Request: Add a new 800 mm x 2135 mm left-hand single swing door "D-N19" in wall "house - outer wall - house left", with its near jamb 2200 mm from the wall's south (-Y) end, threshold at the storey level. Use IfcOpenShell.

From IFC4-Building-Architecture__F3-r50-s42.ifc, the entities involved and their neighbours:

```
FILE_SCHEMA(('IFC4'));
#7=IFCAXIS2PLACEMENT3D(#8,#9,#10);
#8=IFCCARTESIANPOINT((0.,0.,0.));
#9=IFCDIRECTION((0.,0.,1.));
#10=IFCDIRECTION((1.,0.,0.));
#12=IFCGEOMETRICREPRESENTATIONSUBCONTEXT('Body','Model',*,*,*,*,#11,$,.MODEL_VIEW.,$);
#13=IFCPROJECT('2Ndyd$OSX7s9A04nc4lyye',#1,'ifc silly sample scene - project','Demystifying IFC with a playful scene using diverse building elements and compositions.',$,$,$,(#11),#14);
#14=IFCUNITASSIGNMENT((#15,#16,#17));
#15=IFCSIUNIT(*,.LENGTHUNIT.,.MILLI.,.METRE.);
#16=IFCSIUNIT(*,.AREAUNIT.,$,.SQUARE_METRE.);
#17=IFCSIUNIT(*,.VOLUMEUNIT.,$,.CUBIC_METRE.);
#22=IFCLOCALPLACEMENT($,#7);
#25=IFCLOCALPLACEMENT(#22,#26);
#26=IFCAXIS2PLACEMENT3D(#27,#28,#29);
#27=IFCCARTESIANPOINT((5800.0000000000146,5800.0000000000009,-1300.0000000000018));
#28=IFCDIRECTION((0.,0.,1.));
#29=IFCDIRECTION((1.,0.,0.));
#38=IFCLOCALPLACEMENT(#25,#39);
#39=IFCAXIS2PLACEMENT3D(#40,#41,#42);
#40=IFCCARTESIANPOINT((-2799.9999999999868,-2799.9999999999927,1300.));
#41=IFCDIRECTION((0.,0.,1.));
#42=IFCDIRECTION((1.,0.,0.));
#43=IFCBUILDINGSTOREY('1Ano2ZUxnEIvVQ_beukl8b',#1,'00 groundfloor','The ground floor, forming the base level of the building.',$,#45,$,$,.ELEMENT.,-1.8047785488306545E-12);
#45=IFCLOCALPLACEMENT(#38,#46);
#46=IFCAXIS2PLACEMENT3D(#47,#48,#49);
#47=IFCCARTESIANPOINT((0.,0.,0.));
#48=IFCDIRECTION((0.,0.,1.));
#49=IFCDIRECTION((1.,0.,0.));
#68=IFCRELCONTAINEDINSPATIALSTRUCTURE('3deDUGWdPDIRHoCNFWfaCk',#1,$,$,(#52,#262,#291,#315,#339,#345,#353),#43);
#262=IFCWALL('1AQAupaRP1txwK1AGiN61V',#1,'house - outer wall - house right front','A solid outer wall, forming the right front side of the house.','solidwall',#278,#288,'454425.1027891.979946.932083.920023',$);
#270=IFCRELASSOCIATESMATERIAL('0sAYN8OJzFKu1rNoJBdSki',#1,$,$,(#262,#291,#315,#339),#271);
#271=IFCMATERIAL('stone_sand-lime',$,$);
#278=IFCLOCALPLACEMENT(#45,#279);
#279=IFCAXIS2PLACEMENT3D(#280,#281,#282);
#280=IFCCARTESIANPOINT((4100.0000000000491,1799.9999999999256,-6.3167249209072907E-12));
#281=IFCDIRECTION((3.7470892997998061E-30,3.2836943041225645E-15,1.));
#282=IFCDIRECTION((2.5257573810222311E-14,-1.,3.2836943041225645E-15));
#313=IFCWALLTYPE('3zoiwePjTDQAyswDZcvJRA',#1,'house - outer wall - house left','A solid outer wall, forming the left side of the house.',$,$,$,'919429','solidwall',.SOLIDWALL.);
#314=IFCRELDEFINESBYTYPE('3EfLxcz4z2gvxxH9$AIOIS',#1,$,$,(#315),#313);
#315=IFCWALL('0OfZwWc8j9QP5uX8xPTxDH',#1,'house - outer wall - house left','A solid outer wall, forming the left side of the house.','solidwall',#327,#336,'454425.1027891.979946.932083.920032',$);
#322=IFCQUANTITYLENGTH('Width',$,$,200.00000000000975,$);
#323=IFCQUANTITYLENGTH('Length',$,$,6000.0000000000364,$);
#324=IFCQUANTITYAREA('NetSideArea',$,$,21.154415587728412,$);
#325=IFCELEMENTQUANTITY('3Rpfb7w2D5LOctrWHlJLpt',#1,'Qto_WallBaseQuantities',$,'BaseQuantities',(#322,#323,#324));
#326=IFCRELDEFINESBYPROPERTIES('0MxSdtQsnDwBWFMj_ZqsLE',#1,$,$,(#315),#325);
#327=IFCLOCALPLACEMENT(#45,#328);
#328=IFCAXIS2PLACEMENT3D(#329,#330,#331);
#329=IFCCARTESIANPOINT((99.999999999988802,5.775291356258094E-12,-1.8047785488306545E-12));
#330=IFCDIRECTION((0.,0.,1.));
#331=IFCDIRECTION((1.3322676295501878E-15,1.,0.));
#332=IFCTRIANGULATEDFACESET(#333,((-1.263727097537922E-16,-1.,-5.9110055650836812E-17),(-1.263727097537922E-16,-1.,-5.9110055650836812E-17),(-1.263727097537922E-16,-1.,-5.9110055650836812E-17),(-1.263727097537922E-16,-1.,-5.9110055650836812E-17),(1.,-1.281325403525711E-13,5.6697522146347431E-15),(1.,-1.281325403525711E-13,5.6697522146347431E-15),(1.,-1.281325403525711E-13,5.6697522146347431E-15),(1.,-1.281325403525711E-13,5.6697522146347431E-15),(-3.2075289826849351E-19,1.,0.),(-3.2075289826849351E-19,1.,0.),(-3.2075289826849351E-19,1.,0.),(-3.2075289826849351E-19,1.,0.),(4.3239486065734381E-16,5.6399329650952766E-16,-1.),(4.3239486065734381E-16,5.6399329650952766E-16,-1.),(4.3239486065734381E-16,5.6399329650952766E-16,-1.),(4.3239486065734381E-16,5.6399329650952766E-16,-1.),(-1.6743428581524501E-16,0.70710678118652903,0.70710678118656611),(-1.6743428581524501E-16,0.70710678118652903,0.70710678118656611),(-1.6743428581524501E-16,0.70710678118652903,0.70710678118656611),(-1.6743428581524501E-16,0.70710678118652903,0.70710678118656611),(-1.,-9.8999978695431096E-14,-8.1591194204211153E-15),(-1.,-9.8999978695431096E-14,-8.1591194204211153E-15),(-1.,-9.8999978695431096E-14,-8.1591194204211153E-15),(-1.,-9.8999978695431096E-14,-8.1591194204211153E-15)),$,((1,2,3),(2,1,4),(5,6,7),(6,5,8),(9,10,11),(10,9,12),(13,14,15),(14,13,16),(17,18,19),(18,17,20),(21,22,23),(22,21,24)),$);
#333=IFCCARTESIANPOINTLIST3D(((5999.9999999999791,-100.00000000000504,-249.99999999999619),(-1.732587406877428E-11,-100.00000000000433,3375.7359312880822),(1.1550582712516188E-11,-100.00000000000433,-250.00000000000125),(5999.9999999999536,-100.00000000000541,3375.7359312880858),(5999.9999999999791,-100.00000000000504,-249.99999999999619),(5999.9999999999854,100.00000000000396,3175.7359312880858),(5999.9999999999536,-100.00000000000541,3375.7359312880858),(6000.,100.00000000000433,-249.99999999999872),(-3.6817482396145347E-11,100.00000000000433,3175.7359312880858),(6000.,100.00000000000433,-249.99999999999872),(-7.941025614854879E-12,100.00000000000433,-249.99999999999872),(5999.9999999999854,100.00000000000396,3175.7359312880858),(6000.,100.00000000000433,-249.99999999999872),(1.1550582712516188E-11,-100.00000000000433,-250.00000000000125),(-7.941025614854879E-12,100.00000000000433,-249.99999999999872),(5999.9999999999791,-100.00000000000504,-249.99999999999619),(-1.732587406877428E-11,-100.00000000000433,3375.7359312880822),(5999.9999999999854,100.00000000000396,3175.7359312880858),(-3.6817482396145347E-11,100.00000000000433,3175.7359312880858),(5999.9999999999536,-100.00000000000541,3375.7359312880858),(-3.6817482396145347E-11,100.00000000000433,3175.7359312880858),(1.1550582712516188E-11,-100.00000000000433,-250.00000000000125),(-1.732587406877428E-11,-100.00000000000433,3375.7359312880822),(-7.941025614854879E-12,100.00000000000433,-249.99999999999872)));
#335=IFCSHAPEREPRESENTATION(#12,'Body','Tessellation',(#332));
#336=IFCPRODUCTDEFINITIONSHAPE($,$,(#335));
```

```python
import numpy as np
import ifcopenshell
import ifcopenshell.api.feature
import ifcopenshell.api.geometry
import ifcopenshell.api.pset
import ifcopenshell.api.root
import ifcopenshell.api.spatial
import ifcopenshell.geom
import ifcopenshell.util.element
import ifcopenshell.util.placement
import ifcopenshell.util.representation
import ifcopenshell.util.shape
import ifcopenshell.util.unit

model = ifcopenshell.open("IFC4-Building-Architecture__F3-r50-s42.ifc")
unit_scale = ifcopenshell.util.unit.calculate_unit_scale(model)
area_scale = ifcopenshell.util.unit.calculate_unit_scale(model, "AREAUNIT")
settings = ifcopenshell.geom.settings()


def volume(element):
    """Net volume in cubic metres, openings subtracted."""
    shape = ifcopenshell.geom.create_shape(settings, element)
    return ifcopenshell.util.shape.get_volume(shape.geometry)


wall = model.by_guid("0OfZwWc8j9QP5uX8xPTxDH")
storey = ifcopenshell.util.element.get_container(wall, ifc_class="IfcBuildingStorey")
context = ifcopenshell.util.representation.get_context(model, "Model", "Body", "MODEL_VIEW")
before = volume(wall)

width, height, from_end, sill = 0.8, 2.135, 2.2, 0.0  # metres

# The wall runs along its own X axis, and the end named is its -X end.
wall_shape = ifcopenshell.geom.create_shape(settings, wall)
x, y, z = ifcopenshell.util.shape.get_vertices(wall_shape.geometry).T
start = x.min() + from_end
face, thickness = float(y.min()), float(y.max() - y.min())
wall_matrix = ifcopenshell.util.placement.get_local_placement(wall.ObjectPlacement)
level = ifcopenshell.util.placement.get_local_placement(storey.ObjectPlacement)[2, 3]


def in_wall(x, y):
    """Placement at x, y metres in the wall's axes, at sill height."""
    matrix = wall_matrix.copy()
    matrix[:, 3] = wall_matrix @ np.array([x / unit_scale, y / unit_scale, 0.0, 1.0])
    matrix[2, 3] = level + sill / unit_scale
    return matrix


# Opening: a box that overshoots both wall faces by 50 mm.
opening = ifcopenshell.api.root.create_entity(model, ifc_class="IfcOpeningElement", predefined_type="OPENING")
box = ifcopenshell.api.geometry.add_wall_representation(
    model, context=context, length=width, height=height, thickness=thickness + 0.1
)
ifcopenshell.api.geometry.assign_representation(model, product=opening, representation=box)
ifcopenshell.api.geometry.edit_object_placement(model, product=opening, matrix=in_wall(start, face - 0.05), is_si=False)
ifcopenshell.api.feature.add_feature(model, feature=opening, element=wall)

door = ifcopenshell.api.root.create_entity(model, ifc_class="IfcDoor", name="D-N19", predefined_type="DOOR")
door.OverallWidth, door.OverallHeight = width / unit_scale, height / unit_scale
door.OperationType = "SINGLE_SWING_LEFT"
body = ifcopenshell.api.geometry.add_door_representation(
    model,
    context=context,
    overall_width=door.OverallWidth,
    overall_height=door.OverallHeight,
    operation_type="SINGLE_SWING_LEFT",
    lining_properties={"LiningDepth": thickness / unit_scale, "ThresholdDepth": thickness / unit_scale},
)
ifcopenshell.api.geometry.assign_representation(model, product=door, representation=body)
ifcopenshell.api.spatial.assign_container(model, products=[door], relating_structure=storey)
ifcopenshell.api.feature.add_filling(model, opening=opening, element=door)

# The lining spans the wall, so the door starts at the wall face.
ifcopenshell.api.geometry.edit_object_placement(model, product=door, matrix=in_wall(start, face), is_si=False)

after = volume(wall)

# Update the wall's stored quantities.
qto = model.by_id(ifcopenshell.util.element.get_pset(wall, "Qto_WallBaseQuantities", should_inherit=False)["id"])
ifcopenshell.api.pset.edit_qto(model, qto=qto, properties={"NetSideArea": after / thickness / area_scale})

print(f"wall volume {before:.3f} -> {after:.3f} m3")

model.write("IFC4-Building-Architecture__F3-r50-s42-out.ifc")
```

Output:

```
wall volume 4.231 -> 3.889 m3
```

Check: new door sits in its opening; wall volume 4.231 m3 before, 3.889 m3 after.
